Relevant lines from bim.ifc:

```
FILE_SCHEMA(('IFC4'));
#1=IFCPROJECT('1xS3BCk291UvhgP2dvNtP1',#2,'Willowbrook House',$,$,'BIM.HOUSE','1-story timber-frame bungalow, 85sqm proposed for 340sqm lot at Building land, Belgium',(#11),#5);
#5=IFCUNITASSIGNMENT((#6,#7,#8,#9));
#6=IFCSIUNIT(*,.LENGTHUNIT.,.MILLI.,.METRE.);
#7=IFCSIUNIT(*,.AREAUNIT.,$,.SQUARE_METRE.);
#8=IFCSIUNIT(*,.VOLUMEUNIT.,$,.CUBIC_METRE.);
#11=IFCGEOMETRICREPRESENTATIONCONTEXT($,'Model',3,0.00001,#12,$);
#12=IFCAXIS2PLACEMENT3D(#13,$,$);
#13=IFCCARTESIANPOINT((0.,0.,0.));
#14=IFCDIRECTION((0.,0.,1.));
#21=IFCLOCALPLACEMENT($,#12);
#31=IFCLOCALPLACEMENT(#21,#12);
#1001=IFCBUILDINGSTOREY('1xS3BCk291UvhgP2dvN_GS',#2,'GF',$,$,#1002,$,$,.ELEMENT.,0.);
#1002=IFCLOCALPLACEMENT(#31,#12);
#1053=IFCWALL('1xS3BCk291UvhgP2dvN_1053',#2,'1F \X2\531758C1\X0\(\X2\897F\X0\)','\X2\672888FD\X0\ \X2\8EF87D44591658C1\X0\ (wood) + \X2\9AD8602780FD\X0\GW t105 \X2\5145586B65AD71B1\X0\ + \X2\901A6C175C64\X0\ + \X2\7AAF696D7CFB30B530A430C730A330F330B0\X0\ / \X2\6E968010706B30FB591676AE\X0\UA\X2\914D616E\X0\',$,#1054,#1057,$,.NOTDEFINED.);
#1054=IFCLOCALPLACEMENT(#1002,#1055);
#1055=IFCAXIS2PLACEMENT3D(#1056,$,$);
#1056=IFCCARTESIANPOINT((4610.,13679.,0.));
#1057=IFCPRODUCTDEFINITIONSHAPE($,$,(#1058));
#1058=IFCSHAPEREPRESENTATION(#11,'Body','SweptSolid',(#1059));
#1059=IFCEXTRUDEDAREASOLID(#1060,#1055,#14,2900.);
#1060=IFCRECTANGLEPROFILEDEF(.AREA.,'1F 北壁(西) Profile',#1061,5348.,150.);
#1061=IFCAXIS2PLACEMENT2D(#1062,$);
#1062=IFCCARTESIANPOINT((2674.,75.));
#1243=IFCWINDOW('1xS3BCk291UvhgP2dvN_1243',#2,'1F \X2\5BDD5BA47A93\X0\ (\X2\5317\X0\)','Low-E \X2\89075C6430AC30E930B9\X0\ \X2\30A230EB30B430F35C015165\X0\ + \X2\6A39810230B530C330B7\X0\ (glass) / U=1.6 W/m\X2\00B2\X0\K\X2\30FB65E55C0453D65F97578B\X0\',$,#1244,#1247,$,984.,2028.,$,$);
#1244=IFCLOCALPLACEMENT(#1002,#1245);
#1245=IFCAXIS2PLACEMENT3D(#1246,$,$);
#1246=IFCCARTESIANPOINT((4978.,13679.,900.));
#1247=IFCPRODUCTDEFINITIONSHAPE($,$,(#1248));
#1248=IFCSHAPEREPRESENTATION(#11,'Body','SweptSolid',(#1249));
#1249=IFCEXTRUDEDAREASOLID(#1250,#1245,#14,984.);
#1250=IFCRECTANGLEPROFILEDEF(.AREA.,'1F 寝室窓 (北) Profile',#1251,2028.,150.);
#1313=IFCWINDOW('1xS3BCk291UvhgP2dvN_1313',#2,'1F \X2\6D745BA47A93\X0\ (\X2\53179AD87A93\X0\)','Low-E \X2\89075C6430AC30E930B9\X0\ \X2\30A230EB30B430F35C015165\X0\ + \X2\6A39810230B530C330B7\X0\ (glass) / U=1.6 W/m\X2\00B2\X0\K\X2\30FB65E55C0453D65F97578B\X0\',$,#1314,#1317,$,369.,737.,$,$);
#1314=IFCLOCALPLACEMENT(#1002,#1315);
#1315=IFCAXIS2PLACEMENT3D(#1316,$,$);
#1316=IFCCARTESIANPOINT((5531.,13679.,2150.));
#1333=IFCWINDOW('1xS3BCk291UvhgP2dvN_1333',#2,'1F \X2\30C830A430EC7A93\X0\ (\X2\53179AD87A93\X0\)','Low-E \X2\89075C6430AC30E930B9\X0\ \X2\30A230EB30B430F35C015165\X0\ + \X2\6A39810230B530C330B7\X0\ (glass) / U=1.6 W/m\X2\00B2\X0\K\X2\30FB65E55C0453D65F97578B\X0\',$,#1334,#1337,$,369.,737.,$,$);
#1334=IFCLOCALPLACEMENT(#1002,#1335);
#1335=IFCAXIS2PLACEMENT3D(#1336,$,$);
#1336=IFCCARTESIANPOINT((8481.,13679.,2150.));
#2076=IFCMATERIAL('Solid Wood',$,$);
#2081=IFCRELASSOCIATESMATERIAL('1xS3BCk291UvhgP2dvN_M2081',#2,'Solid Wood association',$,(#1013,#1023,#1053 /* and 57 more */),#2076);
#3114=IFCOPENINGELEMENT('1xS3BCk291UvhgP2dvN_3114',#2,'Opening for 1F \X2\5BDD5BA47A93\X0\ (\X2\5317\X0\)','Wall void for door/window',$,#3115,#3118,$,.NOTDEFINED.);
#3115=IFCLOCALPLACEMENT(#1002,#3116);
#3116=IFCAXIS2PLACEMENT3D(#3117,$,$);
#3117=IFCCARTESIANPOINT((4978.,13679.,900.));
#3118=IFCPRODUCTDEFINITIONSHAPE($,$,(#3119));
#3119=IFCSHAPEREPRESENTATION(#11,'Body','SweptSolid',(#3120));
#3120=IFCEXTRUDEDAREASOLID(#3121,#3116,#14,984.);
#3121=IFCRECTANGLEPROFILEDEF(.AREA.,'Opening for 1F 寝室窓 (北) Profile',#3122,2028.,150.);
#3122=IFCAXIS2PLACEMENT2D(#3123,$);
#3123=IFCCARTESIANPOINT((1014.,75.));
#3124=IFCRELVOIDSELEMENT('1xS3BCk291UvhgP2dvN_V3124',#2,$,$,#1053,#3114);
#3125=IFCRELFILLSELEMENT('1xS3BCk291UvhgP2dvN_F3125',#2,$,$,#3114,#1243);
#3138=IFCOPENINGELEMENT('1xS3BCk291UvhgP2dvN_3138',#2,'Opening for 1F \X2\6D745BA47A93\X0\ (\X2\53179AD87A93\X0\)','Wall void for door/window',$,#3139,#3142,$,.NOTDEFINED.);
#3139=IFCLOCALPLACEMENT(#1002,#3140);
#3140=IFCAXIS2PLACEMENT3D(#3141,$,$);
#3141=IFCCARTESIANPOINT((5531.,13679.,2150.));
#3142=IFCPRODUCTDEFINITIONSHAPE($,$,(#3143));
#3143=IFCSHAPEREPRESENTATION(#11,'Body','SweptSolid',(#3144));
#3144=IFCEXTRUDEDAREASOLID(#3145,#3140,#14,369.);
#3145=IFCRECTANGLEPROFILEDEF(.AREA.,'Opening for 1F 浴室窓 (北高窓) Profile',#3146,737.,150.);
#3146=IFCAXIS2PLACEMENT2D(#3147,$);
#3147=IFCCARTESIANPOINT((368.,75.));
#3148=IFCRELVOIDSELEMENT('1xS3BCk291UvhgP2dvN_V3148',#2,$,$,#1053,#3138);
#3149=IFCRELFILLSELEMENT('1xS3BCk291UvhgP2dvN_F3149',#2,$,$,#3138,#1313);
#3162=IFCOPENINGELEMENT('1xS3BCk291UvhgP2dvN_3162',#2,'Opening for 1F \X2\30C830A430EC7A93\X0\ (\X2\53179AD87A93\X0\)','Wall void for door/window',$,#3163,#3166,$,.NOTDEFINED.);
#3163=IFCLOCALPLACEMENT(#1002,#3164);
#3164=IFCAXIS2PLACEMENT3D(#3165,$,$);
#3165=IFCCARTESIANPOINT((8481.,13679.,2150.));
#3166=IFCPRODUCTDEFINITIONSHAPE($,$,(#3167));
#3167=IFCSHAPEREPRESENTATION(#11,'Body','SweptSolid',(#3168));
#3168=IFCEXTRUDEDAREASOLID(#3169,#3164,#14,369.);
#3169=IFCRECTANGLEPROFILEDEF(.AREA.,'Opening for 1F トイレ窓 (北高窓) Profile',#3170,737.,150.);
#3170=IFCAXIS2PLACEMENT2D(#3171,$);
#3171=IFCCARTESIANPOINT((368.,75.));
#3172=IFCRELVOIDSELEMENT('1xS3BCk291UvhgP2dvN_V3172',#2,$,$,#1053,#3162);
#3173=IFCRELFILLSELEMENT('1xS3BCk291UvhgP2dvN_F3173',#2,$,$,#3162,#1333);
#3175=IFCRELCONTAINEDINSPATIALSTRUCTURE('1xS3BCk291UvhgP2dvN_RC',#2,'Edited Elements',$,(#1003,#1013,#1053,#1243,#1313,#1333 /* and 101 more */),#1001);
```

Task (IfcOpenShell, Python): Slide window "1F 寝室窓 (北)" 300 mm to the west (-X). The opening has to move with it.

```python
import ifcopenshell
import ifcopenshell.api.geometry
import ifcopenshell.util.placement
import ifcopenshell.util.unit

model = ifcopenshell.open("bim.ifc")
unit_scale = ifcopenshell.util.unit.calculate_unit_scale(model)

window = model.by_guid("1xS3BCk291UvhgP2dvN_1243")
opening = window.FillsVoids[0].RelatingOpeningElement
wall = opening.VoidsElements[0].RelatingBuildingElement

wall_matrix = ifcopenshell.util.placement.get_local_placement(wall.ObjectPlacement)
shift = wall_matrix[:3, 0] * -0.3 / unit_scale
before = ifcopenshell.util.placement.get_local_placement(window.ObjectPlacement)[:3, 3].copy()

# The window is not placed relative to its opening, so move both.
for product in (opening, window):
    matrix = ifcopenshell.util.placement.get_local_placement(product.ObjectPlacement)
    matrix[:3, 3] += shift
    ifcopenshell.api.geometry.edit_object_placement(model, product=product, matrix=matrix, is_si=False)

after = ifcopenshell.util.placement.get_local_placement(window.ObjectPlacement)[:3, 3]
print("window moved by", (after - before).round(3) + 0.0)

model.write("bim_rev.ifc")
```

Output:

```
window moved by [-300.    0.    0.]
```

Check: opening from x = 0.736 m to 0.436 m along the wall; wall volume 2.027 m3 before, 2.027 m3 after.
